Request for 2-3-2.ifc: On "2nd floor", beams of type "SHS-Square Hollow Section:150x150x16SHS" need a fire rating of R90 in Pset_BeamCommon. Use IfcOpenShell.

First a look at what the model holds.

```python
import ifcopenshell
import ifcopenshell.util.element

model = ifcopenshell.open("2-3-2.ifc")
print(model.schema)
storey = next(s for s in model.by_type("IfcBuildingStorey") if s.Name == "2nd floor")
beams = [e for e in ifcopenshell.util.element.get_decomposition(storey) if e.is_a("IfcBeam")]
seen = {}
for e in beams:
    element_type = ifcopenshell.util.element.get_type(e)
    key = (element_type.Name if element_type != e and element_type else None, ifcopenshell.util.element.get_pset(e, "Pset_BeamCommon", "FireRating"))
    seen[key] = seen.get(key, 0) + 1
for (name, value), count in sorted(seen.items(), key=str):
    print(count, "x", name, "|", value)
```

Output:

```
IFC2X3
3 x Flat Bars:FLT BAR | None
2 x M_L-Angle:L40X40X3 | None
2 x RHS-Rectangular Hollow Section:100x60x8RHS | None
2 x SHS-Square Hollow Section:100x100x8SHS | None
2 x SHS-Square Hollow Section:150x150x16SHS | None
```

```python
import ifcopenshell
import ifcopenshell.api.pset
import ifcopenshell.util.element

model = ifcopenshell.open("2-3-2.ifc")

storey = next(s for s in model.by_type("IfcBuildingStorey") if s.Name == "2nd floor")
beams = [e for e in ifcopenshell.util.element.get_decomposition(storey) if e.is_a("IfcBeam")]

count = 0
for e in beams:
    element_type = ifcopenshell.util.element.get_type(e)
    if element_type in (None, e) or element_type.Name != "SHS-Square Hollow Section:150x150x16SHS":
        continue
    # add_pset returns the element's existing set when there is one.
    pset = ifcopenshell.api.pset.add_pset(model, product=e, name="Pset_BeamCommon")
    ifcopenshell.api.pset.edit_pset(model, pset=pset, properties={"FireRating": "R90"})
    count += 1

print(count, "beams updated")

model.write("2-3-2_edited.ifc")
```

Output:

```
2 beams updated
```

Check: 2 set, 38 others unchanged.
